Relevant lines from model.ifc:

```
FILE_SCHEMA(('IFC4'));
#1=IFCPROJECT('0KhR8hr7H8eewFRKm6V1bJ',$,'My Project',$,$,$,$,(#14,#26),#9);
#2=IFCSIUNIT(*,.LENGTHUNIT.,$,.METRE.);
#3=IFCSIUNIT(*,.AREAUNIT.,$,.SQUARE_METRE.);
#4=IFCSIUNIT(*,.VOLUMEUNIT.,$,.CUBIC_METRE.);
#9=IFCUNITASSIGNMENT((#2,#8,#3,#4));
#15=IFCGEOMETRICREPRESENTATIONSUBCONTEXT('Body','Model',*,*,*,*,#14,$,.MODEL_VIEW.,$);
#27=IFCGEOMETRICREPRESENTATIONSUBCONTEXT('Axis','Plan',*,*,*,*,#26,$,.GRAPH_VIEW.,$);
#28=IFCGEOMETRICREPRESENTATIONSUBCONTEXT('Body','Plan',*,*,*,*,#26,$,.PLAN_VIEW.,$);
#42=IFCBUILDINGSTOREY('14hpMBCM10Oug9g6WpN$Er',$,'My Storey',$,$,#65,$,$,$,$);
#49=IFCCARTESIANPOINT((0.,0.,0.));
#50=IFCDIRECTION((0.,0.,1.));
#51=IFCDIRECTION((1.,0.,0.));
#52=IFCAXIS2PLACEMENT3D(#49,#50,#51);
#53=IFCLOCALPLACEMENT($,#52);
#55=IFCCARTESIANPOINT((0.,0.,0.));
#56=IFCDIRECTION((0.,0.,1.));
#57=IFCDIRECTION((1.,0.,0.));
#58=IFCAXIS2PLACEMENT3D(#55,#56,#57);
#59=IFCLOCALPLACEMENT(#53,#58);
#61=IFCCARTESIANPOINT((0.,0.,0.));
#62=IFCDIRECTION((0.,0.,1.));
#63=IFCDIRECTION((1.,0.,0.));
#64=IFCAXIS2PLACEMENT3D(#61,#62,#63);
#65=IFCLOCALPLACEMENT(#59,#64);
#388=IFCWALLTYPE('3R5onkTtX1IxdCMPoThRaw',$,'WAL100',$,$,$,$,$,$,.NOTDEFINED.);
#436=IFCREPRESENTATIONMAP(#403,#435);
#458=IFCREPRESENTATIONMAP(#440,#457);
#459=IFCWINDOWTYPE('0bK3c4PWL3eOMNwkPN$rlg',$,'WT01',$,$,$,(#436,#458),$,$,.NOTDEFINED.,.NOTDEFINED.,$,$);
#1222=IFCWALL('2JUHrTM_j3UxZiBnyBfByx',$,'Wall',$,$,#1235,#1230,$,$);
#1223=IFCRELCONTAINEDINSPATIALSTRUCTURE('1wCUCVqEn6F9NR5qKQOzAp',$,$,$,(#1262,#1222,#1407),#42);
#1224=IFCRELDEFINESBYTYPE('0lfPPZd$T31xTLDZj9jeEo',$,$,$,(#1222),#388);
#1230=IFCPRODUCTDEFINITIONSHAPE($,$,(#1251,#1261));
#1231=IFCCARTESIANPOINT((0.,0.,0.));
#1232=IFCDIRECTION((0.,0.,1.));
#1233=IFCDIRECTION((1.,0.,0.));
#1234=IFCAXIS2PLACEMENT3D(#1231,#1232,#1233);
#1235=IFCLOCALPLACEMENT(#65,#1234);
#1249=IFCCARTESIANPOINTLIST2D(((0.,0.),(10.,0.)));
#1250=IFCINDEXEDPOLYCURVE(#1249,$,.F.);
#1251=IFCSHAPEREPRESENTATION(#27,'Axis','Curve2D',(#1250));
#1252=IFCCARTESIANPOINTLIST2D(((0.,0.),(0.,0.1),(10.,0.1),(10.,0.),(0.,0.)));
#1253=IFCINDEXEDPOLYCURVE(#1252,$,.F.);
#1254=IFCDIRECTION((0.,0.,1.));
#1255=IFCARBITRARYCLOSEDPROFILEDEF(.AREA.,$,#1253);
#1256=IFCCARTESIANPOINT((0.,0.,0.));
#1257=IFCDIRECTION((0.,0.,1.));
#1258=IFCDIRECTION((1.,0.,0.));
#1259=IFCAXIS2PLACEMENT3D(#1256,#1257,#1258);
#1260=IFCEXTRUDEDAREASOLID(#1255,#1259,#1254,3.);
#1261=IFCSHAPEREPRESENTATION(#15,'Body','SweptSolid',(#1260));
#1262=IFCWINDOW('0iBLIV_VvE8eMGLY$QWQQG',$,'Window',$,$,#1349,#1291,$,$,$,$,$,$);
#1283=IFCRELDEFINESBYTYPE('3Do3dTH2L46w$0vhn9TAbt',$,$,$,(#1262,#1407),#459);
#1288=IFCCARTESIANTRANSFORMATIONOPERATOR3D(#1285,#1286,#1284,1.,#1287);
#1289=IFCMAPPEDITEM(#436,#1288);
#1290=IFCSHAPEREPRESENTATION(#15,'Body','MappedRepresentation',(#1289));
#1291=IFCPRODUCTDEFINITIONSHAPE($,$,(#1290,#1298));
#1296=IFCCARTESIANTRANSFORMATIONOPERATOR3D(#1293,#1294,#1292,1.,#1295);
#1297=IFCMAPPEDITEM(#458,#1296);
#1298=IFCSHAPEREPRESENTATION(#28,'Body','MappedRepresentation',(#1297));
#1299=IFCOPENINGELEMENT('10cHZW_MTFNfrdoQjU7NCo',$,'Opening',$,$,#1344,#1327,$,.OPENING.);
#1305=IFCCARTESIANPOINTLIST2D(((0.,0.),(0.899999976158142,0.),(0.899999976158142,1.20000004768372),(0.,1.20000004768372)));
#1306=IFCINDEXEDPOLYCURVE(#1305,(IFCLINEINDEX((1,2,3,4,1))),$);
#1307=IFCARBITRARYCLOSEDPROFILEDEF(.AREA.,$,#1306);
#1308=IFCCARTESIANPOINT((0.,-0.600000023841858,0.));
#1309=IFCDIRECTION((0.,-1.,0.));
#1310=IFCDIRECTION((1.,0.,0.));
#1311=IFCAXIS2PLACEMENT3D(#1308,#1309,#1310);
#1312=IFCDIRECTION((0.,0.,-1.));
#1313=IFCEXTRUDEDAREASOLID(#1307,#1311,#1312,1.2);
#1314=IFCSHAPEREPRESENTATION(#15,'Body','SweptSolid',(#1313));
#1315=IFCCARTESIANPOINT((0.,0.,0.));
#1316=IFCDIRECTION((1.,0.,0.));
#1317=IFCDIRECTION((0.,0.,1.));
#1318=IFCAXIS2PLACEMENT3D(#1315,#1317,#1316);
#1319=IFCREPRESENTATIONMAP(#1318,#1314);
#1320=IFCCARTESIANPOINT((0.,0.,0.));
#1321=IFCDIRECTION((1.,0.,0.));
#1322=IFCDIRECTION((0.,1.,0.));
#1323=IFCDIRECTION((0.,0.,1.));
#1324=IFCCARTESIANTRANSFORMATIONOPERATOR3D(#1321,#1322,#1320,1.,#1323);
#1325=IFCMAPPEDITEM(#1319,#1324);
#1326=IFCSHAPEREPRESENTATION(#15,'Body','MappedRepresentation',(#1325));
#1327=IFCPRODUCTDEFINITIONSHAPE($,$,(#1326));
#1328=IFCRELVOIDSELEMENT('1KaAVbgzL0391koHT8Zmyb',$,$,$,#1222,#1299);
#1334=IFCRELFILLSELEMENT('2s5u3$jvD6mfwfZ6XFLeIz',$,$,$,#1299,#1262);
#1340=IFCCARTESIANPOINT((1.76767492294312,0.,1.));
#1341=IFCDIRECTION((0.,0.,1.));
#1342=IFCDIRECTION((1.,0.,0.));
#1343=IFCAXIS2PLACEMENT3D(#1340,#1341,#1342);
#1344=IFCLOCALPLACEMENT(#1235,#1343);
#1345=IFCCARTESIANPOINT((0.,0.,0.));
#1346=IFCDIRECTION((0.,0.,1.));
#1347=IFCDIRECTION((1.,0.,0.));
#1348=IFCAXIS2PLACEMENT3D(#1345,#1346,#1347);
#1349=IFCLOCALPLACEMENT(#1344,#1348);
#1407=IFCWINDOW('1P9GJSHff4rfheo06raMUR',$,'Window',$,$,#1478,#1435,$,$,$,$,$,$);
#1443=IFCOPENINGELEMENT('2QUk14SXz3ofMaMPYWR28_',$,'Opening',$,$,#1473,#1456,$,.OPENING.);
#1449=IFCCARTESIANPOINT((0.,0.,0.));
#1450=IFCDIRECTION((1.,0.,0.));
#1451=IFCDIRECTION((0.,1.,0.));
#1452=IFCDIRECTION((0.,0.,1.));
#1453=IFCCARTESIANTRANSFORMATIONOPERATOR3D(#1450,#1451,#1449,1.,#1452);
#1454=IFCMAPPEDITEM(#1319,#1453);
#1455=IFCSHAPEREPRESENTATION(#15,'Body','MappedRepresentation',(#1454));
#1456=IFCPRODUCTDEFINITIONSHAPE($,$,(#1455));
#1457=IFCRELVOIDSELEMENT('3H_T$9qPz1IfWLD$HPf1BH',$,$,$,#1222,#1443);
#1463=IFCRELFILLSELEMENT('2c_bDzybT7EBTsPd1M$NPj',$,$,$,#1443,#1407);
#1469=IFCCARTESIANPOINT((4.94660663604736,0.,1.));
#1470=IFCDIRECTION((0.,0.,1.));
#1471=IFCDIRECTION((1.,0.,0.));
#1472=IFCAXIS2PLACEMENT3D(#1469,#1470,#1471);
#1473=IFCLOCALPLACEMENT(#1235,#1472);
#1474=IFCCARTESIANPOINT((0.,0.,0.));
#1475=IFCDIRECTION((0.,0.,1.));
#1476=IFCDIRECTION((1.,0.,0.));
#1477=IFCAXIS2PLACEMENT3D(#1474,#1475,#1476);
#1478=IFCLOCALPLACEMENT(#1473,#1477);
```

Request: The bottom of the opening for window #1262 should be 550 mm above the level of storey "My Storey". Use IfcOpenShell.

```python
import numpy as np
import ifcopenshell
import ifcopenshell.api.geometry
import ifcopenshell.geom
import ifcopenshell.util.element
import ifcopenshell.util.placement
import ifcopenshell.util.shape
import ifcopenshell.util.unit

model = ifcopenshell.open("model.ifc")
unit_scale = ifcopenshell.util.unit.calculate_unit_scale(model)

window = model.by_guid("0iBLIV_VvE8eMGLY$QWQQG")
opening = window.FillsVoids[0].RelatingOpeningElement
storey = ifcopenshell.util.element.get_container(window, ifc_class="IfcBuildingStorey")
level = ifcopenshell.util.placement.get_local_placement(storey.ObjectPlacement)[2, 3]

# The opening's origin need not be at the sill, so measure its lowest point.
shape = ifcopenshell.geom.create_shape(ifcopenshell.geom.settings(), opening)
bottom = ifcopenshell.util.shape.get_shape_bottom_elevation(shape, shape.geometry) / unit_scale
dz = level + 0.55 / unit_scale - bottom

shift = np.array([0.0, 0.0, dz])
# The window is placed relative to its opening, so it follows when the opening moves.
matrix = ifcopenshell.util.placement.get_local_placement(opening.ObjectPlacement)
matrix[:3, 3] += shift
ifcopenshell.api.geometry.edit_object_placement(
    model, product=opening, matrix=matrix, is_si=False, should_transform_children=True
)

print(f"moved by {dz * unit_scale:+.3f} m")

model.write("model-out.ifc")
```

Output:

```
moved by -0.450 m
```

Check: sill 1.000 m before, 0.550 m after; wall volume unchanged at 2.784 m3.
